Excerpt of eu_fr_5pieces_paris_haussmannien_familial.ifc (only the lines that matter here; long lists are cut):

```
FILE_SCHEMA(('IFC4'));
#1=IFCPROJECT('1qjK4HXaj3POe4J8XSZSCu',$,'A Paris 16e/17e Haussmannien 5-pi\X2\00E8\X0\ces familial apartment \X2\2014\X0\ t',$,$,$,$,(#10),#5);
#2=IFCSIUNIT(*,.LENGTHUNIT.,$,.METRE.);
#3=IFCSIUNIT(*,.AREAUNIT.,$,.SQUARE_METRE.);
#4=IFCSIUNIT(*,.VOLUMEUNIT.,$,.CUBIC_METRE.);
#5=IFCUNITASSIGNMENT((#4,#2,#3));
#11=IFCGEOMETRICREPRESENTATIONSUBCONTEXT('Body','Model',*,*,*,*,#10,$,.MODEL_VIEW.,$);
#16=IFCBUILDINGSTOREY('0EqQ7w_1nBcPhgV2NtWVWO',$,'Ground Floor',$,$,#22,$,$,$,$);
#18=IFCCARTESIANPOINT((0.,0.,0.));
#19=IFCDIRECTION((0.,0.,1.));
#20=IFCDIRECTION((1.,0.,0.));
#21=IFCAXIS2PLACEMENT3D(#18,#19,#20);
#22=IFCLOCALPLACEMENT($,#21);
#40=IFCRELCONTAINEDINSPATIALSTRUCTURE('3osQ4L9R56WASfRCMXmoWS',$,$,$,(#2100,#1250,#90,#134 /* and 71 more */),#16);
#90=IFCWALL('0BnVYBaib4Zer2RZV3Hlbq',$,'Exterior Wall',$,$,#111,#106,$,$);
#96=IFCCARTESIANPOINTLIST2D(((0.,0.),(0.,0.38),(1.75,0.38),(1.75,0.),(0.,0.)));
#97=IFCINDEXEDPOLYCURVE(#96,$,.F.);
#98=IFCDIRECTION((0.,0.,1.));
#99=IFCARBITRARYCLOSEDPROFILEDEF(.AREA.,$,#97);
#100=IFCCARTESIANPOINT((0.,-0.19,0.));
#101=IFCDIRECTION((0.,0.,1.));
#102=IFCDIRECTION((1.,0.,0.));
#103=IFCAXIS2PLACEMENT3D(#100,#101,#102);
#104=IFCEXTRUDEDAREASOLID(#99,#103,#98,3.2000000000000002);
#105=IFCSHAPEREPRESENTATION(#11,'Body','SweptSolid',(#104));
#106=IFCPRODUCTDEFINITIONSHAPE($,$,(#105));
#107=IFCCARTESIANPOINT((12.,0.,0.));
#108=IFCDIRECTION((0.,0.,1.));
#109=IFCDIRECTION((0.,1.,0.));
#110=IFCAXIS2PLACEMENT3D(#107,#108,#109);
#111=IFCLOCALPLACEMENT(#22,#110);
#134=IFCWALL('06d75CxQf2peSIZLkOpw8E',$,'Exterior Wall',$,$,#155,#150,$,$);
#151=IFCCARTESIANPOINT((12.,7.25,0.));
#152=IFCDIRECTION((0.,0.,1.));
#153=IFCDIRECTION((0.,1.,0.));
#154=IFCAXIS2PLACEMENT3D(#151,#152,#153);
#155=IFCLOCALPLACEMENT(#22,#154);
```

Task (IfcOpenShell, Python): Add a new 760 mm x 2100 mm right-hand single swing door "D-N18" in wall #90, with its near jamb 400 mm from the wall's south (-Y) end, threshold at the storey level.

```python
import numpy as np
import ifcopenshell
import ifcopenshell.api.feature
import ifcopenshell.api.geometry
import ifcopenshell.api.root
import ifcopenshell.api.spatial
import ifcopenshell.geom
import ifcopenshell.util.element
import ifcopenshell.util.placement
import ifcopenshell.util.representation
import ifcopenshell.util.shape
import ifcopenshell.util.unit

model = ifcopenshell.open("eu_fr_5pieces_paris_haussmannien_familial.ifc")
unit_scale = ifcopenshell.util.unit.calculate_unit_scale(model)
settings = ifcopenshell.geom.settings()


def volume(element):
    """Net volume in cubic metres, openings subtracted."""
    shape = ifcopenshell.geom.create_shape(settings, element)
    return ifcopenshell.util.shape.get_volume(shape.geometry)


wall = model.by_guid("0BnVYBaib4Zer2RZV3Hlbq")
storey = ifcopenshell.util.element.get_container(wall, ifc_class="IfcBuildingStorey")
context = ifcopenshell.util.representation.get_context(model, "Model", "Body", "MODEL_VIEW")
before = volume(wall)

width, height, from_end, sill = 0.76, 2.1, 0.4, 0.0  # metres

# The wall runs along its own X axis, and the end named is its -X end.
wall_shape = ifcopenshell.geom.create_shape(settings, wall)
x, y, z = ifcopenshell.util.shape.get_vertices(wall_shape.geometry).T
start = x.min() + from_end
face, thickness = float(y.min()), float(y.max() - y.min())
wall_matrix = ifcopenshell.util.placement.get_local_placement(wall.ObjectPlacement)
level = ifcopenshell.util.placement.get_local_placement(storey.ObjectPlacement)[2, 3]


def in_wall(x, y):
    """Placement at x, y metres in the wall's axes, at sill height."""
    matrix = wall_matrix.copy()
    matrix[:, 3] = wall_matrix @ np.array([x / unit_scale, y / unit_scale, 0.0, 1.0])
    matrix[2, 3] = level + sill / unit_scale
    return matrix


# Opening: a box that overshoots both wall faces by 50 mm.
opening = ifcopenshell.api.root.create_entity(model, ifc_class="IfcOpeningElement", predefined_type="OPENING")
box = ifcopenshell.api.geometry.add_wall_representation(
    model, context=context, length=width, height=height, thickness=thickness + 0.1
)
ifcopenshell.api.geometry.assign_representation(model, product=opening, representation=box)
ifcopenshell.api.geometry.edit_object_placement(model, product=opening, matrix=in_wall(start, face - 0.05), is_si=False)
ifcopenshell.api.feature.add_feature(model, feature=opening, element=wall)

door = ifcopenshell.api.root.create_entity(model, ifc_class="IfcDoor", name="D-N18", predefined_type="DOOR")
door.OverallWidth, door.OverallHeight = width / unit_scale, height / unit_scale
door.OperationType = "SINGLE_SWING_RIGHT"
body = ifcopenshell.api.geometry.add_door_representation(
    model,
    context=context,
    overall_width=door.OverallWidth,
    overall_height=door.OverallHeight,
    operation_type="SINGLE_SWING_RIGHT",
    lining_properties={"LiningDepth": thickness / unit_scale, "ThresholdDepth": thickness / unit_scale},
)
ifcopenshell.api.geometry.assign_representation(model, product=door, representation=body)
ifcopenshell.api.spatial.assign_container(model, products=[door], relating_structure=storey)
ifcopenshell.api.feature.add_filling(model, opening=opening, element=door)

# The lining spans the wall, so the door starts at the wall face.
ifcopenshell.api.geometry.edit_object_placement(model, product=door, matrix=in_wall(start, face), is_si=False)

after = volume(wall)

print(f"wall volume {before:.3f} -> {after:.3f} m3")

model.write("eu_fr_5pieces_paris_haussmannien_familial_rev.ifc")
```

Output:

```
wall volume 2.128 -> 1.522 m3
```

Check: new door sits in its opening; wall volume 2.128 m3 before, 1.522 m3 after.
